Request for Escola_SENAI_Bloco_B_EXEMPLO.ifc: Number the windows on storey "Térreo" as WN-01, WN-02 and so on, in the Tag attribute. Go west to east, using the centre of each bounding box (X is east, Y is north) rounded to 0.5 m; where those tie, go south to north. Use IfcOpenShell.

First a look at what the model holds.

```python
import ifcopenshell
import ifcopenshell.util.element
import ifcopenshell.util.placement

model = ifcopenshell.open("Escola_SENAI_Bloco_B_EXEMPLO.ifc")
print(model.schema)
storey = next(s for s in model.by_type("IfcBuildingStorey") if s.Name == "Térreo")
windows = [e for e in ifcopenshell.util.element.get_decomposition(storey) if e.is_a("IfcWindow")]
for e in sorted(windows, key=lambda e: e.id()):
    origin = ifcopenshell.util.placement.get_local_placement(e.ObjectPlacement)[:3, 3]
    print(e.id(), e.Tag, e.Name, origin.round(2) + 0.0, sep=" | ")
```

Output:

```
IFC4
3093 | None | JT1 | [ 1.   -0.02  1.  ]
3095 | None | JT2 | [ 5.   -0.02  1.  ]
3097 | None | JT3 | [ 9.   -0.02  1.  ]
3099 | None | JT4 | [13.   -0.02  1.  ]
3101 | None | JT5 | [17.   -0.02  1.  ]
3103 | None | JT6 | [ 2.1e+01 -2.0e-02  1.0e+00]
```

```python
import ifcopenshell
import ifcopenshell.geom
import ifcopenshell.util.element
import ifcopenshell.util.shape

model = ifcopenshell.open("Escola_SENAI_Bloco_B_EXEMPLO.ifc")
settings = ifcopenshell.geom.settings()
settings.set("use-world-coords", True)


def centre(element):
    shape = ifcopenshell.geom.create_shape(settings, element)
    return ifcopenshell.util.shape.get_bbox_centroid(shape.geometry)


storey = next(s for s in model.by_type("IfcBuildingStorey") if s.Name == "Térreo")
windows = [e for e in ifcopenshell.util.element.get_decomposition(storey) if e.is_a("IfcWindow")]

# Insertion points can sit at a corner or the storey origin, so sort by the geometry (in metres).
centres = {e: centre(e) for e in windows}
windows.sort(key=lambda e: (round(centres[e][0] / 0.5), centres[e][1]))

for i, e in enumerate(windows, start=1):
    number = f"WN-{i:02d}"
    e.Tag = number
    print(e.id(), number)

model.write("Escola_SENAI_Bloco_B_EXEMPLO_v2.ifc")
```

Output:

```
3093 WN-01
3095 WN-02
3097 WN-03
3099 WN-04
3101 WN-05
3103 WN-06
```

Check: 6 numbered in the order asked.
